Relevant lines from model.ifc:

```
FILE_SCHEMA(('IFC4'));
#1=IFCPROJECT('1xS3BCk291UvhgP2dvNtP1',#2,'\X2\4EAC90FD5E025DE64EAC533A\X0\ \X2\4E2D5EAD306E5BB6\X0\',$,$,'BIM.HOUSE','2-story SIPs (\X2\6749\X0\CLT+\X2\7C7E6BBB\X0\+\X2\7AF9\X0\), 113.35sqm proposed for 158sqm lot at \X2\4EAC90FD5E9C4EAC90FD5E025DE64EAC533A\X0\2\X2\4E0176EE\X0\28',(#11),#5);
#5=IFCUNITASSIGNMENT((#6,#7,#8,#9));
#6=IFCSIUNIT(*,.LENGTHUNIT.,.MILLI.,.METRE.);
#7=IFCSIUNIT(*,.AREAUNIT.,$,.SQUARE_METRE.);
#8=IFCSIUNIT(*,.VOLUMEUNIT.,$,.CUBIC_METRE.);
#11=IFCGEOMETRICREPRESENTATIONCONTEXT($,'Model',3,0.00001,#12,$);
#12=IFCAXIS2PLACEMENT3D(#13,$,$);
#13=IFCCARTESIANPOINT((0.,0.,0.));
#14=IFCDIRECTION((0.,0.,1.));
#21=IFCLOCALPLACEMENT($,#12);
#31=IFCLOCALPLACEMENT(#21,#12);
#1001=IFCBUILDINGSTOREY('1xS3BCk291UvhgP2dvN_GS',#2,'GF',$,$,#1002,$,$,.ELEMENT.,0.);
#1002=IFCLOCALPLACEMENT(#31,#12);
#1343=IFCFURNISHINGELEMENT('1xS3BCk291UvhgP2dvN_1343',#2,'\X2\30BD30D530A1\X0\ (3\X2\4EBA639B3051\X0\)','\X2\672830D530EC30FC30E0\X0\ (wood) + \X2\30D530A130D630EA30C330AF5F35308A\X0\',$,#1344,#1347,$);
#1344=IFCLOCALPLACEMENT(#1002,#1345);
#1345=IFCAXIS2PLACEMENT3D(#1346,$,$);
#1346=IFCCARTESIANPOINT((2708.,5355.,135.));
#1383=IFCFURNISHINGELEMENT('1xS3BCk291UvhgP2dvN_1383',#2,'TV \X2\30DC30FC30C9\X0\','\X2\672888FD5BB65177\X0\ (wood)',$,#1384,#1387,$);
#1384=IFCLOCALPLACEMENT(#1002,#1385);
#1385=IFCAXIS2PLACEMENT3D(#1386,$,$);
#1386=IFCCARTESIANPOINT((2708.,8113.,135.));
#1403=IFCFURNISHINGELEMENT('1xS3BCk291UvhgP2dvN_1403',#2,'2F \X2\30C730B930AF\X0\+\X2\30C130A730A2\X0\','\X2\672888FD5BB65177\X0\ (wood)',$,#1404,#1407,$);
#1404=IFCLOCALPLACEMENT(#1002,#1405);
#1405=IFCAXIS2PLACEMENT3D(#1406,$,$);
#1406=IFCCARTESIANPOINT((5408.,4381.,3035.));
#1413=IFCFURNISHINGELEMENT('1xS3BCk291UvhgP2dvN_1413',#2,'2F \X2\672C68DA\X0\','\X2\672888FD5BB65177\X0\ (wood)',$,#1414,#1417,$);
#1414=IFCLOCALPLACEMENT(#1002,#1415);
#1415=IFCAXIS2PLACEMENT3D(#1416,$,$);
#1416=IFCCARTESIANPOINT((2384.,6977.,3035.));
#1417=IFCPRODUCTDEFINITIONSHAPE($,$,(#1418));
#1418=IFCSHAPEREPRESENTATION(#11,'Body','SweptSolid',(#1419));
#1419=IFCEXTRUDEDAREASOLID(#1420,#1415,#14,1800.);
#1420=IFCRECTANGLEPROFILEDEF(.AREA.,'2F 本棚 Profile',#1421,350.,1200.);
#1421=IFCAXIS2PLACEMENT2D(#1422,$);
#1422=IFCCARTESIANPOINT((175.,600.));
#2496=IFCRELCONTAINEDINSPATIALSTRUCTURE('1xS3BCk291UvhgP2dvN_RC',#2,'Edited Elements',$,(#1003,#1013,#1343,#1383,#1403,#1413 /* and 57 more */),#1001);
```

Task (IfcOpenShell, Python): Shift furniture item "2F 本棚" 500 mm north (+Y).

```python
import ifcopenshell
import ifcopenshell.api.geometry
import ifcopenshell.util.placement

model = ifcopenshell.open("model.ifc")

item = model.by_guid("1xS3BCk291UvhgP2dvN_1413")
matrix = ifcopenshell.util.placement.get_local_placement(item.ObjectPlacement)
matrix[1, 3] += 500.0
ifcopenshell.api.geometry.edit_object_placement(model, product=item, matrix=matrix, is_si=False)

print(ifcopenshell.util.placement.get_local_placement(item.ObjectPlacement).round(3) + 0.0)

model.write("model-out.ifc")
```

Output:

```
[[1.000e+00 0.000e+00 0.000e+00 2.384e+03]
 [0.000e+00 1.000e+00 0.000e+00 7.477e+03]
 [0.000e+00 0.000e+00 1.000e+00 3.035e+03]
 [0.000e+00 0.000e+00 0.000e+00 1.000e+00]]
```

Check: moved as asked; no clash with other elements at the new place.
